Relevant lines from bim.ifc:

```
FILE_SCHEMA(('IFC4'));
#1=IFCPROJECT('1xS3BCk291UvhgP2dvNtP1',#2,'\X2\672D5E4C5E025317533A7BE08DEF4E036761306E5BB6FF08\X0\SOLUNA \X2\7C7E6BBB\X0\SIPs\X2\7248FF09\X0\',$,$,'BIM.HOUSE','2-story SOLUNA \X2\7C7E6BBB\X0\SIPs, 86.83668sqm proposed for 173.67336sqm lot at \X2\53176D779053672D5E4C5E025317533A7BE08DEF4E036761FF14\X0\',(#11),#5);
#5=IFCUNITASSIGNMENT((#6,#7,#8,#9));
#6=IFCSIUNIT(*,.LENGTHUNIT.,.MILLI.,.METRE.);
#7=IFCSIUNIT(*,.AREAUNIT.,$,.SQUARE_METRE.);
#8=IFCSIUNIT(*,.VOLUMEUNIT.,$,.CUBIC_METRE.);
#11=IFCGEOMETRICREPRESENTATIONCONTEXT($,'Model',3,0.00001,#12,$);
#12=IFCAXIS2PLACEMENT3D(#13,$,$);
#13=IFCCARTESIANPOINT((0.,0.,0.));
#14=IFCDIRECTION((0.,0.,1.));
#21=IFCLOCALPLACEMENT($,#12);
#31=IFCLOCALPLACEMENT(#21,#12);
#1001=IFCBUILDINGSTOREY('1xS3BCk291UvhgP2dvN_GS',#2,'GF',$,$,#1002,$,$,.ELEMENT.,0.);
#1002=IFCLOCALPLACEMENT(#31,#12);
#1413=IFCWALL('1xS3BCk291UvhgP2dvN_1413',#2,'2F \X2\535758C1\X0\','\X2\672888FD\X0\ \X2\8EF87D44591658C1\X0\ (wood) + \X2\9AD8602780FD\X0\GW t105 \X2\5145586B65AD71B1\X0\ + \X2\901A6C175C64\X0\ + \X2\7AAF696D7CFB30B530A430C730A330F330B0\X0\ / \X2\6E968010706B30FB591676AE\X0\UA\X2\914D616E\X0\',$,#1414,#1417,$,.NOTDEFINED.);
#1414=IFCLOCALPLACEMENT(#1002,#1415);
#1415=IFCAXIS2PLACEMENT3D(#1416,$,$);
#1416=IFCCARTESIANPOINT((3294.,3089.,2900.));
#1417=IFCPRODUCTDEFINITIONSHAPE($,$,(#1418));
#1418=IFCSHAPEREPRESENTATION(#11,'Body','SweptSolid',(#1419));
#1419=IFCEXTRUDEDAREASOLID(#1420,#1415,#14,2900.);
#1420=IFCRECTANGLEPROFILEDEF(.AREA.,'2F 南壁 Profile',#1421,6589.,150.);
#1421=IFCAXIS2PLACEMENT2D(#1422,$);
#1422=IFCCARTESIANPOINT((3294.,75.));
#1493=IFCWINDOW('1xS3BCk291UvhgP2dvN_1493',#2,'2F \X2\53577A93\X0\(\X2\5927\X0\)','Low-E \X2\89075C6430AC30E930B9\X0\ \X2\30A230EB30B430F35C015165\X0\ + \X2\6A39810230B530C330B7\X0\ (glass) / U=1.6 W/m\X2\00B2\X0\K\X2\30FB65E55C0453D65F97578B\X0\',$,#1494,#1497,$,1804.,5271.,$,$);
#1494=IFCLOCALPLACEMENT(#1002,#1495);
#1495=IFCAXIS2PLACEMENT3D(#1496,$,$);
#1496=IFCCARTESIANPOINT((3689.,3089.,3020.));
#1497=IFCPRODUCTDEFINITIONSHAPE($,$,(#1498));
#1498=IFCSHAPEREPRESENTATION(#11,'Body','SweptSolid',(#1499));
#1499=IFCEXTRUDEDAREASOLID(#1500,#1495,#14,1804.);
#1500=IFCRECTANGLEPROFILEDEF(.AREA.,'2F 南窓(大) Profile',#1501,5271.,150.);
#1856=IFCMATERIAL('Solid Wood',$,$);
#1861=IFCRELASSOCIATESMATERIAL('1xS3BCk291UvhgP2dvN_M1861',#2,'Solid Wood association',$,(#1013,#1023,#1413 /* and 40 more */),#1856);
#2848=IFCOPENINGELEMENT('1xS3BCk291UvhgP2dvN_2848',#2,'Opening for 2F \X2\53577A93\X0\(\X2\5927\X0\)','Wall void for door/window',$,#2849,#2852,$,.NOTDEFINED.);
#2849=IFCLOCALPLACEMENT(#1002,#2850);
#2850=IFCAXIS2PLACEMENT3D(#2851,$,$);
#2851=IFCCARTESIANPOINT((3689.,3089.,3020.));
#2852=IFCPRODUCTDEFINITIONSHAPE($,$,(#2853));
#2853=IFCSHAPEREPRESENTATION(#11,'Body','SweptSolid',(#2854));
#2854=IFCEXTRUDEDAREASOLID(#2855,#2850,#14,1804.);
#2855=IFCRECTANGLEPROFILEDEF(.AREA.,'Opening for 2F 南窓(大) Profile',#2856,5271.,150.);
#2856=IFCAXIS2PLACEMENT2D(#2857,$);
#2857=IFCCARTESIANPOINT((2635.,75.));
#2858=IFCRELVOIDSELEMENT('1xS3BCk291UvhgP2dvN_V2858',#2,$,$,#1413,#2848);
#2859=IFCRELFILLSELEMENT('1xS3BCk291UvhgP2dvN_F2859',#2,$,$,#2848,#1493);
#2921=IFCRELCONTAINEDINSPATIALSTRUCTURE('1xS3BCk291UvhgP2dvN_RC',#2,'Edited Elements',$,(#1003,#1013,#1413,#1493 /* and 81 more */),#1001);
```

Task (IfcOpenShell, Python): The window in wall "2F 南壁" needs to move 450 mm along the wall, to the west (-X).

```python
import ifcopenshell
import ifcopenshell.api.geometry
import ifcopenshell.util.placement
import ifcopenshell.util.unit

model = ifcopenshell.open("bim.ifc")
unit_scale = ifcopenshell.util.unit.calculate_unit_scale(model)

window = model.by_guid("1xS3BCk291UvhgP2dvN_1493")
opening = window.FillsVoids[0].RelatingOpeningElement
wall = opening.VoidsElements[0].RelatingBuildingElement

wall_matrix = ifcopenshell.util.placement.get_local_placement(wall.ObjectPlacement)
shift = wall_matrix[:3, 0] * -0.45 / unit_scale
before = ifcopenshell.util.placement.get_local_placement(window.ObjectPlacement)[:3, 3].copy()

# The window is not placed relative to its opening, so move both.
for product in (opening, window):
    matrix = ifcopenshell.util.placement.get_local_placement(product.ObjectPlacement)
    matrix[:3, 3] += shift
    ifcopenshell.api.geometry.edit_object_placement(model, product=product, matrix=matrix, is_si=False)

after = ifcopenshell.util.placement.get_local_placement(window.ObjectPlacement)[:3, 3]
print("window moved by", (after - before).round(3) + 0.0)

model.write("bim_updated.ifc")
```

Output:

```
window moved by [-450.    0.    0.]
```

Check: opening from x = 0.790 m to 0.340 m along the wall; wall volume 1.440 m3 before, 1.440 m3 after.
